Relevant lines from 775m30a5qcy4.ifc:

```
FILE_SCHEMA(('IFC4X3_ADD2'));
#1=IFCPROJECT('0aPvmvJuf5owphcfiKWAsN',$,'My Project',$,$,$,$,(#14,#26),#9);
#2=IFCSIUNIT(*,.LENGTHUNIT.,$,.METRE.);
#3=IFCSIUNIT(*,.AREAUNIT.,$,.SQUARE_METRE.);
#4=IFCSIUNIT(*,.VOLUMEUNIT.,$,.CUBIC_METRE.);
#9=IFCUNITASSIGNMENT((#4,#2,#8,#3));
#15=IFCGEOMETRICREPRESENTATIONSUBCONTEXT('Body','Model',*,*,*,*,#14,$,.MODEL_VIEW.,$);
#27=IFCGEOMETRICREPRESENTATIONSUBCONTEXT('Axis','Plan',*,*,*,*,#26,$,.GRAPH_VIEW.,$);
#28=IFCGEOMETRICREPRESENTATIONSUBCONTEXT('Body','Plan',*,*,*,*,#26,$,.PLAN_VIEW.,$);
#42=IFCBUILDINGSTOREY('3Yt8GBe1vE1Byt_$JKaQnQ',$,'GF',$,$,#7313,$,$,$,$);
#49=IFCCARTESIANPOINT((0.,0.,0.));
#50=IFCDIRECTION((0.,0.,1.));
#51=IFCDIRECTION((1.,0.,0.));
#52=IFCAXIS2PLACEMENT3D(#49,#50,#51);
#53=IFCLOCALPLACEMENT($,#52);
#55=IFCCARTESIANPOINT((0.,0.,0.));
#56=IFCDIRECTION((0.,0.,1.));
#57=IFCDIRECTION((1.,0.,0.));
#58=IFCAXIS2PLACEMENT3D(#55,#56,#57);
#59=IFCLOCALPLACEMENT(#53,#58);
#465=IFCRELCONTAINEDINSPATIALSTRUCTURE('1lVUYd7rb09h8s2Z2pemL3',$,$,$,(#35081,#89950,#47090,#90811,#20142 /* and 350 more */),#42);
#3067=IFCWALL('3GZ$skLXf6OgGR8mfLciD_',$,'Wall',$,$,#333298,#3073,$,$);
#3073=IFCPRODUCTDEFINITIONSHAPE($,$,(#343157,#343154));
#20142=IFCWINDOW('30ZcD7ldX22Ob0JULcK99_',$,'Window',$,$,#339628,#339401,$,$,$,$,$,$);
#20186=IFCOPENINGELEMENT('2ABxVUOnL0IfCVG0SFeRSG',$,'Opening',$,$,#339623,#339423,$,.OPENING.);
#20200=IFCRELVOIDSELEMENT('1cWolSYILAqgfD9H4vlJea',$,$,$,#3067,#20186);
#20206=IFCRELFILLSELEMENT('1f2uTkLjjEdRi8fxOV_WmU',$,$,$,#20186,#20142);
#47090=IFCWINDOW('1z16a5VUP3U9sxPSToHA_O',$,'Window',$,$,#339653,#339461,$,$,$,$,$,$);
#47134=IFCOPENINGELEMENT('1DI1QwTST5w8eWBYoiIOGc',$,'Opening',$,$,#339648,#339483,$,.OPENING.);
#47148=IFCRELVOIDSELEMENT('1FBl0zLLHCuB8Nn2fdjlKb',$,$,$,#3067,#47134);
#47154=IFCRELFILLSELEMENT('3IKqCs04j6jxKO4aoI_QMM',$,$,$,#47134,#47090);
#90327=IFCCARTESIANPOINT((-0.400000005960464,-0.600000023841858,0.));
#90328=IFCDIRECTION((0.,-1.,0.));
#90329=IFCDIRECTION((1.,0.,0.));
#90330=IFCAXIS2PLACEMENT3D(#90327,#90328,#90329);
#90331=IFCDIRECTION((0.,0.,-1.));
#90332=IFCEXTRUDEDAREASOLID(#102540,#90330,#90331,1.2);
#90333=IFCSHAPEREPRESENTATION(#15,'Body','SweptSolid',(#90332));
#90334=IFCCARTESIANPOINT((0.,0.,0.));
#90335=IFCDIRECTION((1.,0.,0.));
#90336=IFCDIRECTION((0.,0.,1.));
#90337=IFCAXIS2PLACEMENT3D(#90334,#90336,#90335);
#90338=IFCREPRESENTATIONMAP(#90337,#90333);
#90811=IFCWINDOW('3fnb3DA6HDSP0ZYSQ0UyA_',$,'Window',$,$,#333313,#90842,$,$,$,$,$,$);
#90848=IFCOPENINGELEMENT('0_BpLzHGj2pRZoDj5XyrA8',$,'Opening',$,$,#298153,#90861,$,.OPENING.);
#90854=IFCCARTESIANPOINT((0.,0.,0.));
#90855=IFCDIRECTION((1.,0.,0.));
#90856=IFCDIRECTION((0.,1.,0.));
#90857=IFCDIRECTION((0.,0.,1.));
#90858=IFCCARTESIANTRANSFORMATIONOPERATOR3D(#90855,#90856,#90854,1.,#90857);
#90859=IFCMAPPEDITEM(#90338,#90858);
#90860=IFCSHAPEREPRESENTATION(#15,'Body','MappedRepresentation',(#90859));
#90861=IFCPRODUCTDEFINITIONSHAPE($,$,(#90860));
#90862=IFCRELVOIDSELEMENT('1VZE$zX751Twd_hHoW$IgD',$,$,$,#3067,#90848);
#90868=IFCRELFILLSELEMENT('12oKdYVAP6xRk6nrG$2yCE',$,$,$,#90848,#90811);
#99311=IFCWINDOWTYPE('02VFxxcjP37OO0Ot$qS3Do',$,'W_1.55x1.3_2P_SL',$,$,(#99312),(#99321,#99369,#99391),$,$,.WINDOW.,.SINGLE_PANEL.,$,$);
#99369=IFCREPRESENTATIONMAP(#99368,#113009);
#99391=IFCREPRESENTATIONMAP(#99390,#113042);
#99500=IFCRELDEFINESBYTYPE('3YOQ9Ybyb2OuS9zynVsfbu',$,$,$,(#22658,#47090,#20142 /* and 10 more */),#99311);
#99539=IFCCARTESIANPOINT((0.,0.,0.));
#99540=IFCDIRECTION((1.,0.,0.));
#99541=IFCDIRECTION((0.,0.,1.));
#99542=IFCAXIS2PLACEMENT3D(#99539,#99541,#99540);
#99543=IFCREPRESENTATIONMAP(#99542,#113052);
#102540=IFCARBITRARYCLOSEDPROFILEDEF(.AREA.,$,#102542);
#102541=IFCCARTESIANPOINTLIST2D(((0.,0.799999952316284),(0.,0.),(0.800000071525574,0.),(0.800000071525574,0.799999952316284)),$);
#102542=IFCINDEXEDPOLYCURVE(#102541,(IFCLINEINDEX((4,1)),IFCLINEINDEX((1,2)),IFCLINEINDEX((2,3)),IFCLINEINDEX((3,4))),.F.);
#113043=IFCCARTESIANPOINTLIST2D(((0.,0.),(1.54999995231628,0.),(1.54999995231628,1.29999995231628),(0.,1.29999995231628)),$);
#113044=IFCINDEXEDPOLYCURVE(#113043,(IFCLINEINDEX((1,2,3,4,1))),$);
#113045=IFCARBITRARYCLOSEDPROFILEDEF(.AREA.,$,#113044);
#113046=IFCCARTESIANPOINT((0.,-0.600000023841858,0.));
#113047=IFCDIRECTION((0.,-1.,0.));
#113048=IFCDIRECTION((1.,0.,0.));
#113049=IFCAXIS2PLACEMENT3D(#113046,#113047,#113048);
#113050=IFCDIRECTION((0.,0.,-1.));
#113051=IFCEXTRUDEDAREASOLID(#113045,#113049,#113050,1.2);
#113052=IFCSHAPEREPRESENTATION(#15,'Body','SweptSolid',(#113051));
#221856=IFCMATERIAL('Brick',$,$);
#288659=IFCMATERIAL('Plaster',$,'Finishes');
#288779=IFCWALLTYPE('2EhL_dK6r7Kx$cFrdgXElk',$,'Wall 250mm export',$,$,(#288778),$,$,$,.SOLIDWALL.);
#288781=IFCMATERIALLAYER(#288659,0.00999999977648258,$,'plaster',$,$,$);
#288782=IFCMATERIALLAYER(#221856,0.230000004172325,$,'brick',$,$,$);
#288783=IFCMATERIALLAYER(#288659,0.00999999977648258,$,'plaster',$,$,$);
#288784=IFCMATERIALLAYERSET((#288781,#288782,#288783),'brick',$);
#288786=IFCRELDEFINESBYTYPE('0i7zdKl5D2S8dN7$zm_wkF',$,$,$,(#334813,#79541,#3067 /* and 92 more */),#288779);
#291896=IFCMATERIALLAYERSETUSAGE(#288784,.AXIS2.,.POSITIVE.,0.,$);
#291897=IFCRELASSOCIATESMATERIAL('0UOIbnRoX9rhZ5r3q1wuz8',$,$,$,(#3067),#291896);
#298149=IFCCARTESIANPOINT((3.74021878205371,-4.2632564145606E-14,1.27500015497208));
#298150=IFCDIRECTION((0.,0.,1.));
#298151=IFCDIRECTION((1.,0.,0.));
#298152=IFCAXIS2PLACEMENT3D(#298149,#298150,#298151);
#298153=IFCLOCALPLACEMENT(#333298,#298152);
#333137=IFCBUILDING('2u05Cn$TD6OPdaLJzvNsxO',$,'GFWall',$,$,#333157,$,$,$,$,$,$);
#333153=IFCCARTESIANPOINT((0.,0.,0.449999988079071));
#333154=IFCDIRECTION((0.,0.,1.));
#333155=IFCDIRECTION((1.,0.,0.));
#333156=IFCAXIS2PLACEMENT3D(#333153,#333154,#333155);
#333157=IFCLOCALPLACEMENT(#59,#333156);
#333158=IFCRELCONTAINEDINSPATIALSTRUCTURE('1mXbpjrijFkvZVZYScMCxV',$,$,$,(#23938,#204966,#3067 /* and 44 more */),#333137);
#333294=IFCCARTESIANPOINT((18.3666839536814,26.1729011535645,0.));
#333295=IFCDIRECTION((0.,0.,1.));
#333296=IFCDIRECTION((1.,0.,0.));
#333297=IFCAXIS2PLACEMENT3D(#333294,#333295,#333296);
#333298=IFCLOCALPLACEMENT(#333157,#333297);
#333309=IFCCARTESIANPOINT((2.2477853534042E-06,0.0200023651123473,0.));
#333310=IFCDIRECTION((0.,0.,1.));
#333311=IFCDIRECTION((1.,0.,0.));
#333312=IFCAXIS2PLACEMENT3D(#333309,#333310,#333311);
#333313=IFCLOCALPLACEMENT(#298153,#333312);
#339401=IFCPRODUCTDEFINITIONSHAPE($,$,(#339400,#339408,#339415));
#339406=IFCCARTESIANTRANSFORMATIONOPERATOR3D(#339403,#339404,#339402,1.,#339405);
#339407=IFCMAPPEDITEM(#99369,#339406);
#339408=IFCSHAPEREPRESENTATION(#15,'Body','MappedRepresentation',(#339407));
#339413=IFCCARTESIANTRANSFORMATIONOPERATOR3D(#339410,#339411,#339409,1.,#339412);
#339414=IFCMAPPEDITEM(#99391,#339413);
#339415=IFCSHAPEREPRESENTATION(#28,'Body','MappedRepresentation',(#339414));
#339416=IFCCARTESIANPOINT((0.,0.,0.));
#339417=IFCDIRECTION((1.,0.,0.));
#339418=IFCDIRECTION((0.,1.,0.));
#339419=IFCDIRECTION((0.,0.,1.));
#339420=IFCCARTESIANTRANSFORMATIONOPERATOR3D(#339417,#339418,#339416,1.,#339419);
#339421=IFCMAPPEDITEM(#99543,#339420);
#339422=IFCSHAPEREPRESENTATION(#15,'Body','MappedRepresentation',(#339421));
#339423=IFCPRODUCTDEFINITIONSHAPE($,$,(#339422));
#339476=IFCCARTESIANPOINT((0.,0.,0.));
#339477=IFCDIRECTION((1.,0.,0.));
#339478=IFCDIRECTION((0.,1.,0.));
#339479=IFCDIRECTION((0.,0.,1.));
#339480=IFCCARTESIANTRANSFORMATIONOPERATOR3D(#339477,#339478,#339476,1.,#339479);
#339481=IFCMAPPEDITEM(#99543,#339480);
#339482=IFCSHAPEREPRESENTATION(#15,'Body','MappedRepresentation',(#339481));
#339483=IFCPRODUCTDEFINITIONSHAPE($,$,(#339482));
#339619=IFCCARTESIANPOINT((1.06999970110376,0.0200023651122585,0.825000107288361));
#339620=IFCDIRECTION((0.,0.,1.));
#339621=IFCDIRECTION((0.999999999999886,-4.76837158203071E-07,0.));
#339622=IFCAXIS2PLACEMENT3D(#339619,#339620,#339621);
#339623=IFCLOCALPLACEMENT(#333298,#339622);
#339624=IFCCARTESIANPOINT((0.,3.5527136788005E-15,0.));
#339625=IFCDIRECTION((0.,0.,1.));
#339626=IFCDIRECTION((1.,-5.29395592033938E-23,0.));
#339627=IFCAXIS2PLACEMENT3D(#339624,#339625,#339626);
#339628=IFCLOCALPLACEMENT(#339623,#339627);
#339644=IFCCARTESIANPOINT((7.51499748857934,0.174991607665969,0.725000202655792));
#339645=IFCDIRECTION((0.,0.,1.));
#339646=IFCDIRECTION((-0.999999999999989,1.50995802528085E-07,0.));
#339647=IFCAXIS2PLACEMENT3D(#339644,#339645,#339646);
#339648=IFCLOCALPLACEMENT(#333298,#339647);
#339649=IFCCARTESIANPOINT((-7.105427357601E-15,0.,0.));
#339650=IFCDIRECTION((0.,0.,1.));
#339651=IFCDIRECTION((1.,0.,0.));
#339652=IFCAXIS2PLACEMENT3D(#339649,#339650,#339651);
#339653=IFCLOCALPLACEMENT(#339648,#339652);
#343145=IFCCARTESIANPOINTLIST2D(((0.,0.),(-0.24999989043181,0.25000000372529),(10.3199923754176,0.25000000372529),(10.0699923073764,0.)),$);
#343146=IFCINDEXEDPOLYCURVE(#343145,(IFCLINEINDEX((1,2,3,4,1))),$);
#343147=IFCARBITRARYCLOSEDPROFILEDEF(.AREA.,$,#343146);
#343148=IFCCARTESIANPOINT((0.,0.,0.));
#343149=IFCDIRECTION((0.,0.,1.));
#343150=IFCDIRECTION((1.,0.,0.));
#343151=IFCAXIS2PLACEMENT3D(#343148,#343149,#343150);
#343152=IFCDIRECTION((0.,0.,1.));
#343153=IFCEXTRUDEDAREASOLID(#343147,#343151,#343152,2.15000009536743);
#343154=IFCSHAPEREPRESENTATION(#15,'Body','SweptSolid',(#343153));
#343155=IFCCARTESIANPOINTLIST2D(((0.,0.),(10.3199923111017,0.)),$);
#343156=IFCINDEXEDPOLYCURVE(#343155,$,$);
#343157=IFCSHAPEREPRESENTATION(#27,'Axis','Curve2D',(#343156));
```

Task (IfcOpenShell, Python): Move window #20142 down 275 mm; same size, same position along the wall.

```python
import numpy as np
import ifcopenshell
import ifcopenshell.api.geometry
import ifcopenshell.util.placement
import ifcopenshell.util.unit

model = ifcopenshell.open("775m30a5qcy4.ifc")
unit_scale = ifcopenshell.util.unit.calculate_unit_scale(model)

window = model.by_guid("30ZcD7ldX22Ob0JULcK99_")
opening = window.FillsVoids[0].RelatingOpeningElement
dz = -0.275

shift = np.array([0.0, 0.0, dz])
# The window is placed relative to its opening, so it follows when the opening moves.
matrix = ifcopenshell.util.placement.get_local_placement(opening.ObjectPlacement)
matrix[:3, 3] += shift
ifcopenshell.api.geometry.edit_object_placement(
    model, product=opening, matrix=matrix, is_si=False, should_transform_children=True
)

print(f"moved by {dz * unit_scale:+.3f} m")

model.write("775m30a5qcy4_updated.ifc")
```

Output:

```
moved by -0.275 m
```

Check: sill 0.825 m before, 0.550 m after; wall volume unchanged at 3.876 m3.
